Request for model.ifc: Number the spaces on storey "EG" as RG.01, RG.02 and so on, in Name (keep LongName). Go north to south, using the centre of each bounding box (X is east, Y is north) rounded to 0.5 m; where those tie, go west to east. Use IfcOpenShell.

First a look at what the model holds.

```python
import ifcopenshell
import ifcopenshell.util.element
import ifcopenshell.util.placement

model = ifcopenshell.open("model.ifc")
print(model.schema)
storey = next(s for s in model.by_type("IfcBuildingStorey") if s.Name == "EG")
spaces = [e for e in ifcopenshell.util.element.get_decomposition(storey) if e.is_a("IfcSpace")]
for e in sorted(spaces, key=lambda e: e.id()):
    origin = ifcopenshell.util.placement.get_local_placement(e.ObjectPlacement)[:3, 3]
    print(e.id(), e.Name, e.LongName, origin.round(2) + 0.0, sep=" | ")
```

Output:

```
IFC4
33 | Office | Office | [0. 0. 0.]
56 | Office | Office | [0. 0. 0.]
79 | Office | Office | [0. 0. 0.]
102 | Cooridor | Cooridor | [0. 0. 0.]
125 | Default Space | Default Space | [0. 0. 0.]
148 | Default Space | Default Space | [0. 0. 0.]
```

```python
import ifcopenshell
import ifcopenshell.geom
import ifcopenshell.util.element
import ifcopenshell.util.shape

model = ifcopenshell.open("model.ifc")
settings = ifcopenshell.geom.settings()
settings.set("use-world-coords", True)


def centre(element):
    shape = ifcopenshell.geom.create_shape(settings, element)
    return ifcopenshell.util.shape.get_bbox_centroid(shape.geometry)


storey = next(s for s in model.by_type("IfcBuildingStorey") if s.Name == "EG")
spaces = [e for e in ifcopenshell.util.element.get_decomposition(storey) if e.is_a("IfcSpace")]

# Insertion points can sit at a corner or the storey origin, so sort by the geometry (in metres).
centres = {e: centre(e) for e in spaces}
spaces.sort(key=lambda e: (-round(centres[e][1] / 0.5), centres[e][0]))

for i, e in enumerate(spaces, start=1):
    number = f"RG.{i:02d}"
    e.Name = number
    print(e.id(), number)

model.write("model-out.ifc")
```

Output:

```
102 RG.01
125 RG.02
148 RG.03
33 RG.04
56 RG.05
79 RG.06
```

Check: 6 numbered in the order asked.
